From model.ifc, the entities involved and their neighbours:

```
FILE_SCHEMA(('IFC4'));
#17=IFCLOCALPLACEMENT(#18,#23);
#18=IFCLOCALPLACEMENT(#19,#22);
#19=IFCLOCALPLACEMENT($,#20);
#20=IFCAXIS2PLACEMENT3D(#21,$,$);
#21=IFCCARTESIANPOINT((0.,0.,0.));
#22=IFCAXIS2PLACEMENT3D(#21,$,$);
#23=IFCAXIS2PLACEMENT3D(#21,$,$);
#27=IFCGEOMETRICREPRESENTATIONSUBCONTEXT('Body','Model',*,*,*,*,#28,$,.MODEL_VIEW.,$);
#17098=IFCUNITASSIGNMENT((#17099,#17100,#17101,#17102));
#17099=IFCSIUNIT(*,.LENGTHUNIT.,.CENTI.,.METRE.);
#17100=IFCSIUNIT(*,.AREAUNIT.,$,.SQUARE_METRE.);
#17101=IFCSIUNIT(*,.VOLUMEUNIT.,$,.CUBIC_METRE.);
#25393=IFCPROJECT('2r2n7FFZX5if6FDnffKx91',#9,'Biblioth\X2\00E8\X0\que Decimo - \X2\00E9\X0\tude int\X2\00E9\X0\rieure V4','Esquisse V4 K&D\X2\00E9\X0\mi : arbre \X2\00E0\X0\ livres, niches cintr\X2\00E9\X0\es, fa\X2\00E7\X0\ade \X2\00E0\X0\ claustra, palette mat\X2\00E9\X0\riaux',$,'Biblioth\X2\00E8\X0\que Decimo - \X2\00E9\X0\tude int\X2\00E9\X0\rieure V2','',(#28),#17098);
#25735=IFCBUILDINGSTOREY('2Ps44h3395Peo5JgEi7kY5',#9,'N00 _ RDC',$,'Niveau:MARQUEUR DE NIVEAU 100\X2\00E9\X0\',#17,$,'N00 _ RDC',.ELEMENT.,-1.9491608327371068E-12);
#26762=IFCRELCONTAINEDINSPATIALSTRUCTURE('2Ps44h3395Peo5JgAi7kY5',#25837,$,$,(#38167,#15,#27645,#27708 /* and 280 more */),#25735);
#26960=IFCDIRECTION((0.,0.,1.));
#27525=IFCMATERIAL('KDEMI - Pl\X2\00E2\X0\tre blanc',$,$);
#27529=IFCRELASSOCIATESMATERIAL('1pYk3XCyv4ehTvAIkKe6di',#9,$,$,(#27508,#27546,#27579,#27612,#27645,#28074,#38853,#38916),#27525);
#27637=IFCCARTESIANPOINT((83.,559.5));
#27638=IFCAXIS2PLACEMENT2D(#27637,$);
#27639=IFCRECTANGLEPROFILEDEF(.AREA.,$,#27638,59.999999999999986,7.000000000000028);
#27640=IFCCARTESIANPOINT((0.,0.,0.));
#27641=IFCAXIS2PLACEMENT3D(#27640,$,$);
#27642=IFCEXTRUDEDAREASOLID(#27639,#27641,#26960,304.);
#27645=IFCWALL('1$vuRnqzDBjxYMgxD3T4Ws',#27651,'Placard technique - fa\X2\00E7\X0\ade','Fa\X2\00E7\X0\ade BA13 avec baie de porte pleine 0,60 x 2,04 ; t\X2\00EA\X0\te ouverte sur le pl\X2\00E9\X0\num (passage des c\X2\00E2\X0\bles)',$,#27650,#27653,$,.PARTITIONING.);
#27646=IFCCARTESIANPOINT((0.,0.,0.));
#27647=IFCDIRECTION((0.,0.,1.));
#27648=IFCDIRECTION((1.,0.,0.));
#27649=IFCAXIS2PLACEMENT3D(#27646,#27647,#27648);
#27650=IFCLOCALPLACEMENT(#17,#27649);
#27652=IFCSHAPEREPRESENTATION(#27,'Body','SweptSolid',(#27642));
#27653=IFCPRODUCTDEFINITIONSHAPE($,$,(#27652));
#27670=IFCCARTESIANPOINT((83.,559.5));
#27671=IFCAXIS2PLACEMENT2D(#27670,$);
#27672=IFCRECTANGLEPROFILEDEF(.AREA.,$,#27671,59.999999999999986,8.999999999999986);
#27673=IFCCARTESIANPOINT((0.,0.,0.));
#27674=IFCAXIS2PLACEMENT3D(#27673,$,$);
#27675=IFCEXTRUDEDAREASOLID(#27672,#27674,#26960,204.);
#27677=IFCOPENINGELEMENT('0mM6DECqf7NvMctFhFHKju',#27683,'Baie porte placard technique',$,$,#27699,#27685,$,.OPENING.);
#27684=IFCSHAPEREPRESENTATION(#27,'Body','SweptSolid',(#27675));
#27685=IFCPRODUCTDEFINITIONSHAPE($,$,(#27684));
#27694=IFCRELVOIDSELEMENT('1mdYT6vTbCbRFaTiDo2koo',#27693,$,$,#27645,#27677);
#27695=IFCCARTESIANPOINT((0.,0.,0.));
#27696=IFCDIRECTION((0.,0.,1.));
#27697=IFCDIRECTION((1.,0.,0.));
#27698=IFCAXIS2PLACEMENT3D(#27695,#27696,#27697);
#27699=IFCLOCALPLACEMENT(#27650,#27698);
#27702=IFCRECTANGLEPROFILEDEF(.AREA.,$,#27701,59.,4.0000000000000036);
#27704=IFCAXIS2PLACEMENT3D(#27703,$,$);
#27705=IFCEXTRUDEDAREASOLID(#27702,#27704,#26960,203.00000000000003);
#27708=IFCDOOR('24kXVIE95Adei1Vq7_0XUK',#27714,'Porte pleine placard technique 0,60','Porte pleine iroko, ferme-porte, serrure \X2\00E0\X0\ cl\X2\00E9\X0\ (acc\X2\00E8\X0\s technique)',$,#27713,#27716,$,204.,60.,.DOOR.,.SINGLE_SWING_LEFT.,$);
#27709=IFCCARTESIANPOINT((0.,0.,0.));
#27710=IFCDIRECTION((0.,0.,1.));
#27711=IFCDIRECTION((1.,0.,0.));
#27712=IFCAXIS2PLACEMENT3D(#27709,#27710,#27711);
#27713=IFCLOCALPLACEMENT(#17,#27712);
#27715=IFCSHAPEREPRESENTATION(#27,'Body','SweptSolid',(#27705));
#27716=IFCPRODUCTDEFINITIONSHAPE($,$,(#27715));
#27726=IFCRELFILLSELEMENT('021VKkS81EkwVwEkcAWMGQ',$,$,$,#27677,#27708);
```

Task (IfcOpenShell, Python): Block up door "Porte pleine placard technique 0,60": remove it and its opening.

```python
import ifcopenshell
import ifcopenshell.api.feature
import ifcopenshell.api.root
import ifcopenshell.geom
import ifcopenshell.util.shape

model = ifcopenshell.open("model.ifc")
settings = ifcopenshell.geom.settings()


def volume(element):
    """Net volume in cubic metres, openings subtracted."""
    shape = ifcopenshell.geom.create_shape(settings, element)
    return ifcopenshell.util.shape.get_volume(shape.geometry)


door = model.by_id(27708)
opening = door.FillsVoids[0].RelatingOpeningElement
wall = opening.VoidsElements[0].RelatingBuildingElement
before = volume(wall)

ifcopenshell.api.root.remove_product(model, product=door)
ifcopenshell.api.feature.remove_feature(model, feature=opening)

after = volume(wall)

print(f"wall volume {before:.3f} -> {after:.3f} m3")

model.write("model_rev.ifc")
```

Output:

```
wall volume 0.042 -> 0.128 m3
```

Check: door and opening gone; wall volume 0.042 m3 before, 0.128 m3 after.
